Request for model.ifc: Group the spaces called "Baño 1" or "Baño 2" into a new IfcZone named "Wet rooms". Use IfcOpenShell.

First a look at what the model holds.

```python
import ifcopenshell

model = ifcopenshell.open("model.ifc")
print(model.schema)
seen = {}
for space in model.by_type("IfcSpace"):
    seen[space.LongName] = seen.get(space.LongName, 0) + 1
for name, count in sorted(seen.items(), key=str):
    print(count, "x", name)
print("zones:", [z.Name for z in model.by_type("IfcZone")][:20])
```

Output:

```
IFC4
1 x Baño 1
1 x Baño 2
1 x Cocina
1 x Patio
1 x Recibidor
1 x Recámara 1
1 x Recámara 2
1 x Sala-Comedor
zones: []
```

```python
import ifcopenshell
import ifcopenshell.api.group
import ifcopenshell.api.root

model = ifcopenshell.open("model.ifc")

names = {"Baño 1", "Baño 2"}
spaces = [s for s in model.by_type("IfcSpace") if s.LongName in names]

zone = ifcopenshell.api.root.create_entity(model, ifc_class="IfcZone", name="Wet rooms")
ifcopenshell.api.group.assign_group(model, products=spaces, group=zone)
print(len(spaces), "spaces in", zone.Name)

model.write("model_rev.ifc")
```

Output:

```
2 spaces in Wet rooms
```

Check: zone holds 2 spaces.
